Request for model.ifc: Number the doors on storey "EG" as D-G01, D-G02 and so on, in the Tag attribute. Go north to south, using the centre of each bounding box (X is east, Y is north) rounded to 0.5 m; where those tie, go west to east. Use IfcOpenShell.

First a look at what the model holds.

```python
import ifcopenshell
import ifcopenshell.util.element
import ifcopenshell.util.placement

model = ifcopenshell.open("model.ifc")
print(model.schema)
storey = next(s for s in model.by_type("IfcBuildingStorey") if s.Name == "EG")
doors = [e for e in ifcopenshell.util.element.get_decomposition(storey) if e.is_a("IfcDoor")]
for e in sorted(doors, key=lambda e: e.id()):
    origin = ifcopenshell.util.placement.get_local_placement(e.ObjectPlacement)[:3, 3]
    print(e.id(), e.Tag, e.Name, origin.round(2) + 0.0, sep=" | ")
```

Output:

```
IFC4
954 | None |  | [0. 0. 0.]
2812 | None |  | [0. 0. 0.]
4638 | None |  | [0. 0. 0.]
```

```python
import ifcopenshell
import ifcopenshell.geom
import ifcopenshell.util.element
import ifcopenshell.util.shape

model = ifcopenshell.open("model.ifc")
settings = ifcopenshell.geom.settings()
settings.set("use-world-coords", True)


def centre(element):
    shape = ifcopenshell.geom.create_shape(settings, element)
    return ifcopenshell.util.shape.get_bbox_centroid(shape.geometry)


storey = next(s for s in model.by_type("IfcBuildingStorey") if s.Name == "EG")
doors = [e for e in ifcopenshell.util.element.get_decomposition(storey) if e.is_a("IfcDoor")]

# Insertion points can sit at a corner or the storey origin, so sort by the geometry (in metres).
centres = {e: centre(e) for e in doors}
doors.sort(key=lambda e: (-round(centres[e][1] / 0.5), centres[e][0]))

for i, e in enumerate(doors, start=1):
    number = f"D-G{i:02d}"
    e.Tag = number
    print(e.id(), number)

model.write("model-out.ifc")
```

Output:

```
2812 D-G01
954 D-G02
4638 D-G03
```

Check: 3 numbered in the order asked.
